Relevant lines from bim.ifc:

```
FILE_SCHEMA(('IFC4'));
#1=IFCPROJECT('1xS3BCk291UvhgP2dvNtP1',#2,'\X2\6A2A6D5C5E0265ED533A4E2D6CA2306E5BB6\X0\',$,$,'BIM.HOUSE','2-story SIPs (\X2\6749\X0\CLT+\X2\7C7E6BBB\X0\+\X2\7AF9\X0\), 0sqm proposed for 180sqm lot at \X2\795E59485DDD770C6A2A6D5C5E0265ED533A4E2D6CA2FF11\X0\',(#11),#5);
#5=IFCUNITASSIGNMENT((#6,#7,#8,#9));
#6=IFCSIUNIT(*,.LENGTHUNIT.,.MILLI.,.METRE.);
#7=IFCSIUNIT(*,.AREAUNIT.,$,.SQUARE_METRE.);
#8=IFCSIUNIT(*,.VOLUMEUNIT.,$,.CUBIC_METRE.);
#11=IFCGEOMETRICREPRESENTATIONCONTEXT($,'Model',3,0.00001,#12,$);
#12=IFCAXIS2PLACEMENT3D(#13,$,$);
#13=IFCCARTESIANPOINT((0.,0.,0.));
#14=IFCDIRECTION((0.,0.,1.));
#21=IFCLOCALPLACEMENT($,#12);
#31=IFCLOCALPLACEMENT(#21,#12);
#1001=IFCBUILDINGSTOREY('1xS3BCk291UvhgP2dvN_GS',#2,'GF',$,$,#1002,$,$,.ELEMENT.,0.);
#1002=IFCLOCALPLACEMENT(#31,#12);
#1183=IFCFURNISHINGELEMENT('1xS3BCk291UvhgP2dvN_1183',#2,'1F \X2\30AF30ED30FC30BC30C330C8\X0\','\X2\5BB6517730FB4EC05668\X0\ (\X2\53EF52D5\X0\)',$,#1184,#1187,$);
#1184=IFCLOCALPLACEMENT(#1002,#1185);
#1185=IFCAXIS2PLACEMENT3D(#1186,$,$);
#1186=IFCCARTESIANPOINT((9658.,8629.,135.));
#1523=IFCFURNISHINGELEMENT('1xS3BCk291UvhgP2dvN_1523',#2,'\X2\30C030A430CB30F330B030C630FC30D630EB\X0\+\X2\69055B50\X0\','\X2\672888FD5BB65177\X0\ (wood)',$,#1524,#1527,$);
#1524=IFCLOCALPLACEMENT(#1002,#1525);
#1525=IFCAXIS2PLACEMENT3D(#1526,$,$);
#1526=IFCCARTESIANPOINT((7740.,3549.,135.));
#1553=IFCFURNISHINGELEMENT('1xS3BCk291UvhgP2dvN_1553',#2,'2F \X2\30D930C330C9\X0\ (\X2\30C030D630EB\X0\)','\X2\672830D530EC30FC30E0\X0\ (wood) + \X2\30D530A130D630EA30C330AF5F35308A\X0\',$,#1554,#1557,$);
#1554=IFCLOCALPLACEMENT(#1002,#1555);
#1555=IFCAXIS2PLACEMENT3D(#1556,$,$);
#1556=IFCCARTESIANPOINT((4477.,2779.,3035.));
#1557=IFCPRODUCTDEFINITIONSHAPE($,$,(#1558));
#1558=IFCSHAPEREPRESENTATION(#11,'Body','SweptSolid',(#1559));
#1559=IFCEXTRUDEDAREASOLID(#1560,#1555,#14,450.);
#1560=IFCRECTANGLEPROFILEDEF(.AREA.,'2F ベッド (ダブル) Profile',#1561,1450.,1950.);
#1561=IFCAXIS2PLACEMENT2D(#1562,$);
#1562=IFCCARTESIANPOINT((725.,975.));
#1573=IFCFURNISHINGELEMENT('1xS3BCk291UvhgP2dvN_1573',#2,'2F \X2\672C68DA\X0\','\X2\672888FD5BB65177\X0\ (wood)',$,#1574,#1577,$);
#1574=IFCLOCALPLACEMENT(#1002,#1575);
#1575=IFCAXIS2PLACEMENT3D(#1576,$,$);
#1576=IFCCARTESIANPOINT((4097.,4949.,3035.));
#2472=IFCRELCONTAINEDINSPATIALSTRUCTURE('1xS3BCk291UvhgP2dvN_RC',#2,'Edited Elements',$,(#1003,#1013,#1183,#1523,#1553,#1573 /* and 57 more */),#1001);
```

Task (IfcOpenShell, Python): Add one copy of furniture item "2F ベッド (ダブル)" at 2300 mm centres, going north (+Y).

```python
import numpy as np
import ifcopenshell
import ifcopenshell.api.geometry
import ifcopenshell.api.root
import ifcopenshell.util.element
import ifcopenshell.util.placement
import ifcopenshell.util.unit

model = ifcopenshell.open("bim.ifc")
unit_scale = ifcopenshell.util.unit.calculate_unit_scale(model)


def reuse_history(source, copy):
    """copy_class also copies each property set's owner history, people and application; keep the originals."""
    for rel in copy.IsDefinedBy:
        if rel.is_a("IfcRelDefinesByProperties") and (history := rel.RelatingPropertyDefinition.OwnerHistory):
            rel.RelatingPropertyDefinition.OwnerHistory = source.OwnerHistory
            ifcopenshell.util.element.remove_deep2(model, history)


source = model.by_guid("1xS3BCk291UvhgP2dvN_1553")
base = ifcopenshell.util.placement.get_local_placement(source.ObjectPlacement)
step = np.array([0.0, 1.0, 0.0]) * 2.3 / unit_scale

for i in range(1, 2):
    copy = ifcopenshell.api.root.copy_class(model, product=source)
    copy.Representation = ifcopenshell.util.element.copy_deep(
        model, source.Representation, exclude=["IfcGeometricRepresentationContext", "IfcRepresentationMap"]
    )
    reuse_history(source, copy)
    matrix = base.copy()
    matrix[:3, 3] += i * step
    print("added at", matrix[:3, 3].round(3) + 0.0)
    ifcopenshell.api.geometry.edit_object_placement(model, product=copy, matrix=matrix, is_si=False)

model.write("bim_v2.ifc")
```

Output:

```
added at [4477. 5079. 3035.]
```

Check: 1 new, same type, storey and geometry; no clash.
